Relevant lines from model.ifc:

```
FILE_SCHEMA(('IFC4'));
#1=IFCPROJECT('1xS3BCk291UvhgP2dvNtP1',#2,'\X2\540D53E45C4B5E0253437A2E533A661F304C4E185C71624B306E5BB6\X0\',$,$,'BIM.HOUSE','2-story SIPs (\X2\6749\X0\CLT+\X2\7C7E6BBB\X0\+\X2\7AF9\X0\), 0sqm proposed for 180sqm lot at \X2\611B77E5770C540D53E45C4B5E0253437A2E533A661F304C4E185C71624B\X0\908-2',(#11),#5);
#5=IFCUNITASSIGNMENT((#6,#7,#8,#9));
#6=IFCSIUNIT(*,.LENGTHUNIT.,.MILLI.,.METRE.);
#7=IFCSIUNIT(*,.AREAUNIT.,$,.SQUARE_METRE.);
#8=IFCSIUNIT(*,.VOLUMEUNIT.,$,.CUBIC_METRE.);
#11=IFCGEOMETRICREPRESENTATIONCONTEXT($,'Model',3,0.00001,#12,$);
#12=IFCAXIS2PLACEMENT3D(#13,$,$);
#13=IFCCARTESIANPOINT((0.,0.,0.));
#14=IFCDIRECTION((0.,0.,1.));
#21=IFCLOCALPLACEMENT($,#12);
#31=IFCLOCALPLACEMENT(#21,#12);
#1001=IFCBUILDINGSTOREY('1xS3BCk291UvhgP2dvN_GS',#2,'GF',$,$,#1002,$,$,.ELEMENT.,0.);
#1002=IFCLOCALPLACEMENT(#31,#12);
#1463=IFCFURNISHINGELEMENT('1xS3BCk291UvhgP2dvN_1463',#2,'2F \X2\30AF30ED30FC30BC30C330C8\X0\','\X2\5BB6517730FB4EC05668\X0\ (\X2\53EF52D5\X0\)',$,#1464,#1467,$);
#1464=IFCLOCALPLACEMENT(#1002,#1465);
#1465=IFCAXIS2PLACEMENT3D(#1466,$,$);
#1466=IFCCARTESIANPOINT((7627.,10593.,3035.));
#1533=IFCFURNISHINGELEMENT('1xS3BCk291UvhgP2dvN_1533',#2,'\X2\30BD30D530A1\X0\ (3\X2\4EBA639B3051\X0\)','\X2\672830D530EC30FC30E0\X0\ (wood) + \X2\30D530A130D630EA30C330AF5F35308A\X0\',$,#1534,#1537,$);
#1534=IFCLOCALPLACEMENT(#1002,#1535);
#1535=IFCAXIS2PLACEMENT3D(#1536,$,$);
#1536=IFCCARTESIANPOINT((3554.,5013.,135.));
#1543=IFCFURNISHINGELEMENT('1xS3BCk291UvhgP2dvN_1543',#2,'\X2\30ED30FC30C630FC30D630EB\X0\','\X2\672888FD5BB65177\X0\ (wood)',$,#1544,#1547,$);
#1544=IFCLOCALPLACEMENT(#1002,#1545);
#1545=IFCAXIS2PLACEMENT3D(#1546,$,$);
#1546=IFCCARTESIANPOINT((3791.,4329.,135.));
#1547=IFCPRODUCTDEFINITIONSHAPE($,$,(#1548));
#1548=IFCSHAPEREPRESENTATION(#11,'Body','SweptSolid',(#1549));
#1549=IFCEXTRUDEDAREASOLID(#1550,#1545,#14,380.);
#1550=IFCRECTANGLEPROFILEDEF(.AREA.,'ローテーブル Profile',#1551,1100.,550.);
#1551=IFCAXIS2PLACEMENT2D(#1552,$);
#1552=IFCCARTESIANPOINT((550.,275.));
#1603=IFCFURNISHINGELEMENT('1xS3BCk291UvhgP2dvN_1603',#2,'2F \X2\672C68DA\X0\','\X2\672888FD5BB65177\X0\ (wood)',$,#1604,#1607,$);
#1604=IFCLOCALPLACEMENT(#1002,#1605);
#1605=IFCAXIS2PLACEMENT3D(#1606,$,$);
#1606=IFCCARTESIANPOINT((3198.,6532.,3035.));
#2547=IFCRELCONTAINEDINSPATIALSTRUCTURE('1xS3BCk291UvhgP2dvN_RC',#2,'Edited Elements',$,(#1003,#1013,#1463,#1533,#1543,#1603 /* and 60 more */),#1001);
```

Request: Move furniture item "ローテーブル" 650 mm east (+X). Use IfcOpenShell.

```python
import ifcopenshell
import ifcopenshell.api.geometry
import ifcopenshell.util.placement
import ifcopenshell.util.unit

model = ifcopenshell.open("model.ifc")
unit_scale = ifcopenshell.util.unit.calculate_unit_scale(model)

item = model.by_guid("1xS3BCk291UvhgP2dvN_1543")
matrix = ifcopenshell.util.placement.get_local_placement(item.ObjectPlacement)
matrix[0, 3] += 0.65 / unit_scale
ifcopenshell.api.geometry.edit_object_placement(model, product=item, matrix=matrix, is_si=False)

print(ifcopenshell.util.placement.get_local_placement(item.ObjectPlacement).round(3) + 0.0)

model.write("model-out.ifc")
```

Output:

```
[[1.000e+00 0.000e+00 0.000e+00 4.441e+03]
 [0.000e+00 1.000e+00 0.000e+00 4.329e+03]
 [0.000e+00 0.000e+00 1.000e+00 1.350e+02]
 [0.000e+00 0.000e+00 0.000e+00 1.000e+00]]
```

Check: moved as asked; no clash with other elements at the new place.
